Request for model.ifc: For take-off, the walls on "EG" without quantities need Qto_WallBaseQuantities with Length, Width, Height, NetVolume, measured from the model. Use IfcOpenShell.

First a look at what the model holds.

```python
import ifcopenshell
import ifcopenshell.util.element
import ifcopenshell.util.unit

model = ifcopenshell.open("model.ifc")
print(model.schema)
for unit_type in ("LENGTHUNIT", "AREAUNIT", "VOLUMEUNIT"):
    print(unit_type, ifcopenshell.util.unit.calculate_unit_scale(model, unit_type))
storey = next(s for s in model.by_type("IfcBuildingStorey") if s.Name == "EG")
walls = [e for e in ifcopenshell.util.element.get_decomposition(storey) if e.is_a("IfcWall")]
for e in sorted(walls, key=lambda e: e.id()):
    print(e.id(), e.is_a(), e.Name, list(ifcopenshell.util.element.get_psets(e, qtos_only=True)), sep=" | ")
```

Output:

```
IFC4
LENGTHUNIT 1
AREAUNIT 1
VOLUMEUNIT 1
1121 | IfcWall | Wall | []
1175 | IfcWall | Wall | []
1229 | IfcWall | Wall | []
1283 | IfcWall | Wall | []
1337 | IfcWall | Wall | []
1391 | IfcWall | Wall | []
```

```python
import ifcopenshell
import ifcopenshell.api.pset
import ifcopenshell.geom
import ifcopenshell.util.element
import ifcopenshell.util.shape
import ifcopenshell.util.unit

model = ifcopenshell.open("model.ifc")
unit_scale = ifcopenshell.util.unit.calculate_unit_scale(model)
volume_scale = ifcopenshell.util.unit.calculate_unit_scale(model, "VOLUMEUNIT")
settings = ifcopenshell.geom.settings()

storey = next(s for s in model.by_type("IfcBuildingStorey") if s.Name == "EG")
walls = [e for e in ifcopenshell.util.element.get_decomposition(storey) if e.is_a("IfcWall")]

for e in sorted(walls, key=lambda e: e.id()):
    if ifcopenshell.util.element.get_psets(e, qtos_only=True, should_inherit=False):
        continue
    # Geometry comes back in metres, in the element's own axes.
    shape = ifcopenshell.geom.create_shape(settings, e)
    values = {
        "Length": ifcopenshell.util.shape.get_x(shape.geometry) / unit_scale,
        "Width": ifcopenshell.util.shape.get_y(shape.geometry) / unit_scale,
        "Height": ifcopenshell.util.shape.get_z(shape.geometry) / unit_scale,
        "NetVolume": ifcopenshell.util.shape.get_volume(shape.geometry) / volume_scale,
    }
    qto = ifcopenshell.api.pset.add_qto(model, product=e, name="Qto_WallBaseQuantities")
    ifcopenshell.api.pset.edit_qto(model, qto=qto, properties=values)
    print(e.id(), {k: round(v, 3) for k, v in values.items()})

model.write("model-out.ifc")
```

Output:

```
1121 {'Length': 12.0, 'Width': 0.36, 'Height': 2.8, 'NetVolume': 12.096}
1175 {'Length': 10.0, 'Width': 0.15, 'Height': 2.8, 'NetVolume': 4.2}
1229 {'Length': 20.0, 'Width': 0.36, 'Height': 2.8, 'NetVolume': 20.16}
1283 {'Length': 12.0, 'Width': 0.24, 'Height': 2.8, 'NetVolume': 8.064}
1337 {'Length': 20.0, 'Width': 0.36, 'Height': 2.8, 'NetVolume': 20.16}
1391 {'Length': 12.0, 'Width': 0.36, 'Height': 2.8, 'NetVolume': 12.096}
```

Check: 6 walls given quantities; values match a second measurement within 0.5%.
